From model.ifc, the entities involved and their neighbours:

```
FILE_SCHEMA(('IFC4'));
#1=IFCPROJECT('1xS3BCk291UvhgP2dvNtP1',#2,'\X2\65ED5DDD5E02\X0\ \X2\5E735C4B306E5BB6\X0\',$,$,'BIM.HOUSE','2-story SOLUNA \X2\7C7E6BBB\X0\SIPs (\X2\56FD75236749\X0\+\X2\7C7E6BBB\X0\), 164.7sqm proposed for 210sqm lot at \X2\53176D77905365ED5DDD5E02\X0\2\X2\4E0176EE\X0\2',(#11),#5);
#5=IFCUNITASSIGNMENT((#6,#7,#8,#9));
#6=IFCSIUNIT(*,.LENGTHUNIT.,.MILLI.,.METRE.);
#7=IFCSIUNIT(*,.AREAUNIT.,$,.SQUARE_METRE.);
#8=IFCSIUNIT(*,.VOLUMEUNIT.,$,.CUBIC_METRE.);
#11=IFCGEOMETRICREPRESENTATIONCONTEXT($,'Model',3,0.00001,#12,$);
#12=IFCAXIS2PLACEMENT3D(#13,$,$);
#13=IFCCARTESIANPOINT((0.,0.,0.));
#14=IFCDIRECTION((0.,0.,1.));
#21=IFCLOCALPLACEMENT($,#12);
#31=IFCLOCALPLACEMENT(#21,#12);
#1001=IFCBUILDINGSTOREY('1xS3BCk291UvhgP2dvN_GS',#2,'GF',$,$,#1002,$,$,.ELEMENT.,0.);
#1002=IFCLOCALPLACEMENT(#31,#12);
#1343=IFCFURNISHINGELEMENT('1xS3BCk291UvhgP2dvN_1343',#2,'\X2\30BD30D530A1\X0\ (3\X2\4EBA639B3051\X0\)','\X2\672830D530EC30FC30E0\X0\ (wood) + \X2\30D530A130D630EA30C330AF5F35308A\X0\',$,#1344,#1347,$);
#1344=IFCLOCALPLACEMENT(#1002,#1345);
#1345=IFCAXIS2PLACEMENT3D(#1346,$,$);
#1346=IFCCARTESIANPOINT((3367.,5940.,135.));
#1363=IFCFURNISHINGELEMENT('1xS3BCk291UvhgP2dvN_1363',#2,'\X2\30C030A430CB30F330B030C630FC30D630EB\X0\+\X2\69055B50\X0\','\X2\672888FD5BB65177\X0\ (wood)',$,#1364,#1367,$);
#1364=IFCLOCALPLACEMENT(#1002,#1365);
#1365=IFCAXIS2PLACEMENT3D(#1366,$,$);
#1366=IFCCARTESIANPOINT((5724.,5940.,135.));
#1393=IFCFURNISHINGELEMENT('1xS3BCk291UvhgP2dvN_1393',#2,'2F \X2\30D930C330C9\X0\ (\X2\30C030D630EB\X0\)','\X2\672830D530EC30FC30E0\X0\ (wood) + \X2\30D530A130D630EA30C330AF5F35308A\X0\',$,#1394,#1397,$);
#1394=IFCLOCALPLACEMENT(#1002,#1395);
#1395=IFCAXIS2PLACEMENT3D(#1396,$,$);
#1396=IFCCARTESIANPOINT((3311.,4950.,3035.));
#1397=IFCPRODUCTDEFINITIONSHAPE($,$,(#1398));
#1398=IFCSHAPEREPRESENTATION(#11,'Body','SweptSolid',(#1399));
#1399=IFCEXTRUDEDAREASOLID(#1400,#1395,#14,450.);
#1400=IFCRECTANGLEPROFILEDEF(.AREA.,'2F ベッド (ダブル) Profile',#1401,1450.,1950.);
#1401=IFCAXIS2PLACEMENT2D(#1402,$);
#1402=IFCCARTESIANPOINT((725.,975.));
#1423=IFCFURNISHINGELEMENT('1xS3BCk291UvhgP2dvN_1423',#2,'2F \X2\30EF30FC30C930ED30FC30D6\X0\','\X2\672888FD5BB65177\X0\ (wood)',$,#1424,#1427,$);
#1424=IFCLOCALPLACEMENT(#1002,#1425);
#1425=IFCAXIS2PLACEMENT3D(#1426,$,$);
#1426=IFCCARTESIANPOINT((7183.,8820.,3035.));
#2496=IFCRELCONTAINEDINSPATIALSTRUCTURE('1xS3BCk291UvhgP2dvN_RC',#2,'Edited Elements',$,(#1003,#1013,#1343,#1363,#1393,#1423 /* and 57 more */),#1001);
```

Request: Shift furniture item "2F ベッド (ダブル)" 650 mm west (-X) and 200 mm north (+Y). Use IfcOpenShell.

```python
import ifcopenshell
import ifcopenshell.api.geometry
import ifcopenshell.util.placement

model = ifcopenshell.open("model.ifc")

item = model.by_guid("1xS3BCk291UvhgP2dvN_1393")
matrix = ifcopenshell.util.placement.get_local_placement(item.ObjectPlacement)
matrix[0, 3] -= 650.0
matrix[1, 3] += 200.0
ifcopenshell.api.geometry.edit_object_placement(model, product=item, matrix=matrix, is_si=False)

print(ifcopenshell.util.placement.get_local_placement(item.ObjectPlacement).round(3) + 0.0)

model.write("model_updated.ifc")
```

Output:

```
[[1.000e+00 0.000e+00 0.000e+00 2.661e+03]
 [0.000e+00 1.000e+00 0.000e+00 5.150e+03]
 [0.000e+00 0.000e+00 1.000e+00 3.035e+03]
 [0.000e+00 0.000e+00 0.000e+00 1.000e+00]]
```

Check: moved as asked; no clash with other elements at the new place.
